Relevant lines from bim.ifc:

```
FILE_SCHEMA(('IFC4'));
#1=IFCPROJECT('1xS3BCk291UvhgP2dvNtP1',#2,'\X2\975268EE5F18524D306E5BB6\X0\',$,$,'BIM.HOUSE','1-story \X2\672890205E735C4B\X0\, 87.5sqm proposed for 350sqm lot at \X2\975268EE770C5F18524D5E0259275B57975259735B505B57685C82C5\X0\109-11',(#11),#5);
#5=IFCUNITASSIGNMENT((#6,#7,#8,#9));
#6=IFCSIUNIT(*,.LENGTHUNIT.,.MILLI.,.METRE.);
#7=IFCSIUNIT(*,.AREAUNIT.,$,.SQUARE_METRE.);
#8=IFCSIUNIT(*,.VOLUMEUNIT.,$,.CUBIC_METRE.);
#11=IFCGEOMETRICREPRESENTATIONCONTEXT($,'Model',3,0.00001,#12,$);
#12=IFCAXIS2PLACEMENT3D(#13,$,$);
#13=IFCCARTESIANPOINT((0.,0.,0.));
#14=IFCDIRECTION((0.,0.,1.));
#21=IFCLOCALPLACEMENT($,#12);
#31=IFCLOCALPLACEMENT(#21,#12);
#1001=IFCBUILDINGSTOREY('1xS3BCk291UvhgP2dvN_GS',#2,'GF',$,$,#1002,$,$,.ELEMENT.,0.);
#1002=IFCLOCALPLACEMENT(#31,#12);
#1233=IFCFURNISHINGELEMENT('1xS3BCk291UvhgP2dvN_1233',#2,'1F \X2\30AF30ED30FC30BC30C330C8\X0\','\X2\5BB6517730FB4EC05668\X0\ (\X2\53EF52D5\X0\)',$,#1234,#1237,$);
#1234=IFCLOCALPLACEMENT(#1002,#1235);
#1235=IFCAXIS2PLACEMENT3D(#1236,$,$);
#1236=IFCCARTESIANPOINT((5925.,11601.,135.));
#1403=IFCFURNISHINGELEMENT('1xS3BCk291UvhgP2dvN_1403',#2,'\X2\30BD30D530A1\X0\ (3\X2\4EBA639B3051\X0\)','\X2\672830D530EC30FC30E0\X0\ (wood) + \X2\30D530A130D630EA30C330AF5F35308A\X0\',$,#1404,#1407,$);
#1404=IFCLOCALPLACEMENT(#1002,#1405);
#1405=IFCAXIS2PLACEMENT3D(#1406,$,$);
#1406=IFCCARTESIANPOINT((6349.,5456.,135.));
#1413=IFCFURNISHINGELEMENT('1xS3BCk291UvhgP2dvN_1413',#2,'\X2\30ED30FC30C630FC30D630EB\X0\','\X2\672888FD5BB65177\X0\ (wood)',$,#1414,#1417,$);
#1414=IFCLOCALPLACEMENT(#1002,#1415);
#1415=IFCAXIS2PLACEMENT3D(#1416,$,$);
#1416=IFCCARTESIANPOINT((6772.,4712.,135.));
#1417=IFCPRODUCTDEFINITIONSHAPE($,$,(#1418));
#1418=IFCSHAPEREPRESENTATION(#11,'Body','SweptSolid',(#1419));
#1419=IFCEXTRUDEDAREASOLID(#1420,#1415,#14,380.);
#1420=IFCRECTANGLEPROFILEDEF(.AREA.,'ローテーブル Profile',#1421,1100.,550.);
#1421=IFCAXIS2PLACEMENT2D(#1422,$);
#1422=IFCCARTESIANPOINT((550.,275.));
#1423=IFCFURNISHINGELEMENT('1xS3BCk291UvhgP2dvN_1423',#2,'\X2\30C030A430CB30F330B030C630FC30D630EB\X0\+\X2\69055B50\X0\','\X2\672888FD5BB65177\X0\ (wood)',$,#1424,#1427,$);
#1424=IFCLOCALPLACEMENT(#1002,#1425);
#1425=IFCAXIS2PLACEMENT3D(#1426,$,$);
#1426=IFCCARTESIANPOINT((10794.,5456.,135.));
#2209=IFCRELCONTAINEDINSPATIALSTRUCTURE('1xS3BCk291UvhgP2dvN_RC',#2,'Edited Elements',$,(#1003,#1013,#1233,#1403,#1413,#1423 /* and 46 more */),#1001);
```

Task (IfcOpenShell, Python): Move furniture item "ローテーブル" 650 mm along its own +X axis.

```python
import ifcopenshell
import ifcopenshell.api.geometry
import ifcopenshell.util.placement
import ifcopenshell.util.unit

model = ifcopenshell.open("bim.ifc")
unit_scale = ifcopenshell.util.unit.calculate_unit_scale(model)

item = model.by_guid("1xS3BCk291UvhgP2dvN_1413")
matrix = ifcopenshell.util.placement.get_local_placement(item.ObjectPlacement)
matrix[:3, 3] += matrix[:3, 0] * 0.65 / unit_scale
ifcopenshell.api.geometry.edit_object_placement(model, product=item, matrix=matrix, is_si=False)

print(ifcopenshell.util.placement.get_local_placement(item.ObjectPlacement).round(3) + 0.0)

model.write("bim_edited.ifc")
```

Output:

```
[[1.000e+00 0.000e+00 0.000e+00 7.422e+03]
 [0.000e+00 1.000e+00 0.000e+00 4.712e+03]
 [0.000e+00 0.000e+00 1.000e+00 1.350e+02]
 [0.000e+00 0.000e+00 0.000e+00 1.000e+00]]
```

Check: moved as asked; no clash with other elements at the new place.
